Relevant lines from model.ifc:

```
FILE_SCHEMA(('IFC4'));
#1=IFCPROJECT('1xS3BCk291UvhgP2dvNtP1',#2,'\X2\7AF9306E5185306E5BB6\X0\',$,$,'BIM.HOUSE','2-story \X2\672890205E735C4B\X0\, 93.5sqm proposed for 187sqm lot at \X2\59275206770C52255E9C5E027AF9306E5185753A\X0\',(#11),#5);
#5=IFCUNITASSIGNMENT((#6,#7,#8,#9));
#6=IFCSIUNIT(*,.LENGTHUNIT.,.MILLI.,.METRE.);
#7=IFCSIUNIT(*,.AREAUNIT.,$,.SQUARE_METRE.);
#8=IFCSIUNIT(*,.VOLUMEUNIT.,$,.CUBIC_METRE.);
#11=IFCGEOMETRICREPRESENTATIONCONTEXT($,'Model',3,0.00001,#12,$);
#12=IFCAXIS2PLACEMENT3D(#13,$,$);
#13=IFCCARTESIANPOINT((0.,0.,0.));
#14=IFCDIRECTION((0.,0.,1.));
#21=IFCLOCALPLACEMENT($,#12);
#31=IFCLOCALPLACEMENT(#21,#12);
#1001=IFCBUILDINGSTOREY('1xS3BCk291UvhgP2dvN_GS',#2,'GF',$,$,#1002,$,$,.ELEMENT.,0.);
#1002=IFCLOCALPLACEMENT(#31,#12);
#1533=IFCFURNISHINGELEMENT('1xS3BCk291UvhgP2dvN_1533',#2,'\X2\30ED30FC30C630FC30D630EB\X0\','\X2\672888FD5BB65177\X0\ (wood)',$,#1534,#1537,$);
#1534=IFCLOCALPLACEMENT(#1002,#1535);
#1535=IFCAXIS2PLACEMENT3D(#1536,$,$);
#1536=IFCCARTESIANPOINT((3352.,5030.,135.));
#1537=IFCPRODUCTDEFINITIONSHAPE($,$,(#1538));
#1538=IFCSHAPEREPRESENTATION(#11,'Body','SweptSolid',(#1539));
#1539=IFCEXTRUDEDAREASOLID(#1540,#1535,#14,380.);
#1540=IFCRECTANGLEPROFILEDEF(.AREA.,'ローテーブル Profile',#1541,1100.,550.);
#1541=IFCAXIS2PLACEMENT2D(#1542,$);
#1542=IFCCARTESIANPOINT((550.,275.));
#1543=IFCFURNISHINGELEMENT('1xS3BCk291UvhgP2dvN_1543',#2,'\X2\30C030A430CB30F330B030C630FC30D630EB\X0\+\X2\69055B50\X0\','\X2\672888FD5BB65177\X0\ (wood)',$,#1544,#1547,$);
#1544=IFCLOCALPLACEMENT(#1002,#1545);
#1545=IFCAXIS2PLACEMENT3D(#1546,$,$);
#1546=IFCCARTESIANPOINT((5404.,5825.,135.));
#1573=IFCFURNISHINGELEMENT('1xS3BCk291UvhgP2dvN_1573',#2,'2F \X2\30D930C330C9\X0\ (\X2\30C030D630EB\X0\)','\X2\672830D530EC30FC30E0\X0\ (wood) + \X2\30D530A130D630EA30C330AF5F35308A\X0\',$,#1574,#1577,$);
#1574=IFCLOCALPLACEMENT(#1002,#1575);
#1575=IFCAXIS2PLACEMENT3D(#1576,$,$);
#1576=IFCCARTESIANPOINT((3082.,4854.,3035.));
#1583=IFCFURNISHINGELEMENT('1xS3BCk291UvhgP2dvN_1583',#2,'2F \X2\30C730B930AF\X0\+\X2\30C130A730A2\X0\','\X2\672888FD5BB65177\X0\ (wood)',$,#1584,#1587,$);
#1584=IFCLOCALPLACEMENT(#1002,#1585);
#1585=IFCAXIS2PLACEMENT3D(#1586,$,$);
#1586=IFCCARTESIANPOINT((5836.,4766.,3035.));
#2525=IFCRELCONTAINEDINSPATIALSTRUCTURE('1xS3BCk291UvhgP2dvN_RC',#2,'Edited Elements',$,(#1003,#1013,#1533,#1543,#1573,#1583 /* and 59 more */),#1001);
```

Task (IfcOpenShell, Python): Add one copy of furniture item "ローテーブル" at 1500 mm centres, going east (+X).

```python
import numpy as np
import ifcopenshell
import ifcopenshell.api.geometry
import ifcopenshell.api.root
import ifcopenshell.util.element
import ifcopenshell.util.placement
import ifcopenshell.util.unit

model = ifcopenshell.open("model.ifc")
unit_scale = ifcopenshell.util.unit.calculate_unit_scale(model)


def reuse_history(source, copy):
    """copy_class also copies each property set's owner history, people and application; keep the originals."""
    for rel in copy.IsDefinedBy:
        if rel.is_a("IfcRelDefinesByProperties") and (history := rel.RelatingPropertyDefinition.OwnerHistory):
            rel.RelatingPropertyDefinition.OwnerHistory = source.OwnerHistory
            ifcopenshell.util.element.remove_deep2(model, history)


source = model.by_id(1533)
base = ifcopenshell.util.placement.get_local_placement(source.ObjectPlacement)
step = np.array([1.0, 0.0, 0.0]) * 1.5 / unit_scale

for i in range(1, 2):
    copy = ifcopenshell.api.root.copy_class(model, product=source)
    copy.Representation = ifcopenshell.util.element.copy_deep(
        model, source.Representation, exclude=["IfcGeometricRepresentationContext", "IfcRepresentationMap"]
    )
    reuse_history(source, copy)
    matrix = base.copy()
    matrix[:3, 3] += i * step
    print("added at", matrix[:3, 3].round(3) + 0.0)
    ifcopenshell.api.geometry.edit_object_placement(model, product=copy, matrix=matrix, is_si=False)

model.write("model_v2.ifc")
```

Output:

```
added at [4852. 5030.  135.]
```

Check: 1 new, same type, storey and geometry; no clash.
